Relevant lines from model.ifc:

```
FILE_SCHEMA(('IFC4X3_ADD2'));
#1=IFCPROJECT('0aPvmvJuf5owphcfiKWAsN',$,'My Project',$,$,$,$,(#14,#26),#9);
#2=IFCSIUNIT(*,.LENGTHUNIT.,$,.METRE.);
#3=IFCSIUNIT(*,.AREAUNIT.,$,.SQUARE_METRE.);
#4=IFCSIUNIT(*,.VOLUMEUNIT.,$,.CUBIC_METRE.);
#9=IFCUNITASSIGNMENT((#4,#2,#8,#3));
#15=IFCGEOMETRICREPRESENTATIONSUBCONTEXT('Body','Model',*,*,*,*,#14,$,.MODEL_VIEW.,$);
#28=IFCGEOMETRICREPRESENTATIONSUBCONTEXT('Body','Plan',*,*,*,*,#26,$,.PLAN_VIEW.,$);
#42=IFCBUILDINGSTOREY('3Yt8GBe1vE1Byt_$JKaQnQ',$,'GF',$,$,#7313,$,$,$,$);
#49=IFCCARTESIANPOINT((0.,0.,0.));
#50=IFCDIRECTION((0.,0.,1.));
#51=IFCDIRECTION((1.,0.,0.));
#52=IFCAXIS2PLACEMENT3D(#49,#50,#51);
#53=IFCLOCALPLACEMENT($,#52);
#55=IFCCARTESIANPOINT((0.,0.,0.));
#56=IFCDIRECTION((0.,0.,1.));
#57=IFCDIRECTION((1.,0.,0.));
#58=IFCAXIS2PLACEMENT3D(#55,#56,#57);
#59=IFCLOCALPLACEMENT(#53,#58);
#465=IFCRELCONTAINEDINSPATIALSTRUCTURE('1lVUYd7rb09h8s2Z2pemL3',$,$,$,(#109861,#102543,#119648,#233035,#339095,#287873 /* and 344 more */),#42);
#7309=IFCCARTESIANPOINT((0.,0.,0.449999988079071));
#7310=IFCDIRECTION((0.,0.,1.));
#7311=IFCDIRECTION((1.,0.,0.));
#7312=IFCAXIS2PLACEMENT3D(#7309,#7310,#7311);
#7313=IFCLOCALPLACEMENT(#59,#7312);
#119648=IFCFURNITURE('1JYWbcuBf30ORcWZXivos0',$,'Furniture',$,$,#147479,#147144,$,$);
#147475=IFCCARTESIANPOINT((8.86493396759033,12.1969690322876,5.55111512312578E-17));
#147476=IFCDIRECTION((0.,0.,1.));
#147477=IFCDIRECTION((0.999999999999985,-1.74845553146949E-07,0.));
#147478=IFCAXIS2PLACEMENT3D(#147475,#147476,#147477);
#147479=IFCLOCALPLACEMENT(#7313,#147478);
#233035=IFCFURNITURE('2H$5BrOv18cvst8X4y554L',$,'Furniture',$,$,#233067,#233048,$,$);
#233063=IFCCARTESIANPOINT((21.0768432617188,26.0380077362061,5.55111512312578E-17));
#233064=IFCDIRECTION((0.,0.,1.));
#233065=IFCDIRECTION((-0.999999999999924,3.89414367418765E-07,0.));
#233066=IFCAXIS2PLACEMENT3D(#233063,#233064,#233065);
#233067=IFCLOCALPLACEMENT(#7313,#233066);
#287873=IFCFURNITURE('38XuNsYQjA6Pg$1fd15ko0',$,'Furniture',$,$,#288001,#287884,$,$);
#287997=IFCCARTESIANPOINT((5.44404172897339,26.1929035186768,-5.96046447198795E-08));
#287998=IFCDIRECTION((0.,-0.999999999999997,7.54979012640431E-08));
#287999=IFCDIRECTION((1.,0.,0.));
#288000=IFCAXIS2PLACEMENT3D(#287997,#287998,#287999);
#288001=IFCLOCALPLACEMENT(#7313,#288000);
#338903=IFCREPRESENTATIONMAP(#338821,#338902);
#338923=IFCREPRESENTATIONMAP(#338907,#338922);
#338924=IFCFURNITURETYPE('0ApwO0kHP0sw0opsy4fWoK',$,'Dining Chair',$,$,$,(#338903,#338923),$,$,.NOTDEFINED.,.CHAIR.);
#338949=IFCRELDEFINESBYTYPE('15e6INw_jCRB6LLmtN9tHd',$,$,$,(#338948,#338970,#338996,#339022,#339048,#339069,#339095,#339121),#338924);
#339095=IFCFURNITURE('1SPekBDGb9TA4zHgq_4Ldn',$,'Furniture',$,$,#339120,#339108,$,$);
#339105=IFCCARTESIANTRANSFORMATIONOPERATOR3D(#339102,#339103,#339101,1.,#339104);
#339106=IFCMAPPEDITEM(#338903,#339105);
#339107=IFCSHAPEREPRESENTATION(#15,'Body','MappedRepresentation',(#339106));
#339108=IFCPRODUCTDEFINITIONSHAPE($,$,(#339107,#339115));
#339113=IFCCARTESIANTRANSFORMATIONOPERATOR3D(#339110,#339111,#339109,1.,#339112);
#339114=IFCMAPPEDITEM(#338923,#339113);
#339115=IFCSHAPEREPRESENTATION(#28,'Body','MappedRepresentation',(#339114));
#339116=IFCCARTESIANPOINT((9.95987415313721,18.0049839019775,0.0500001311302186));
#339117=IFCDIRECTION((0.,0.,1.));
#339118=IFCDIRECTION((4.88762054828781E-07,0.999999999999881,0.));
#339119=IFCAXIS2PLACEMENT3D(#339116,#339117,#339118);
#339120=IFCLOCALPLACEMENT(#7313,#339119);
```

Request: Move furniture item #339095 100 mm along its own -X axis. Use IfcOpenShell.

```python
import ifcopenshell
import ifcopenshell.api.geometry
import ifcopenshell.util.placement
import ifcopenshell.util.unit

model = ifcopenshell.open("model.ifc")
unit_scale = ifcopenshell.util.unit.calculate_unit_scale(model)

item = model.by_id(339095)
matrix = ifcopenshell.util.placement.get_local_placement(item.ObjectPlacement)
matrix[:3, 3] -= matrix[:3, 0] * 0.1 / unit_scale
ifcopenshell.api.geometry.edit_object_placement(model, product=item, matrix=matrix, is_si=False)

print(ifcopenshell.util.placement.get_local_placement(item.ObjectPlacement).round(3) + 0.0)

model.write("model_edited.ifc")
```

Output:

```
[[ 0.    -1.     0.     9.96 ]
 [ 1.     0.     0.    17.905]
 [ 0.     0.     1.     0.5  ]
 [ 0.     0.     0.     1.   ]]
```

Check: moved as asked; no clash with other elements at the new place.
